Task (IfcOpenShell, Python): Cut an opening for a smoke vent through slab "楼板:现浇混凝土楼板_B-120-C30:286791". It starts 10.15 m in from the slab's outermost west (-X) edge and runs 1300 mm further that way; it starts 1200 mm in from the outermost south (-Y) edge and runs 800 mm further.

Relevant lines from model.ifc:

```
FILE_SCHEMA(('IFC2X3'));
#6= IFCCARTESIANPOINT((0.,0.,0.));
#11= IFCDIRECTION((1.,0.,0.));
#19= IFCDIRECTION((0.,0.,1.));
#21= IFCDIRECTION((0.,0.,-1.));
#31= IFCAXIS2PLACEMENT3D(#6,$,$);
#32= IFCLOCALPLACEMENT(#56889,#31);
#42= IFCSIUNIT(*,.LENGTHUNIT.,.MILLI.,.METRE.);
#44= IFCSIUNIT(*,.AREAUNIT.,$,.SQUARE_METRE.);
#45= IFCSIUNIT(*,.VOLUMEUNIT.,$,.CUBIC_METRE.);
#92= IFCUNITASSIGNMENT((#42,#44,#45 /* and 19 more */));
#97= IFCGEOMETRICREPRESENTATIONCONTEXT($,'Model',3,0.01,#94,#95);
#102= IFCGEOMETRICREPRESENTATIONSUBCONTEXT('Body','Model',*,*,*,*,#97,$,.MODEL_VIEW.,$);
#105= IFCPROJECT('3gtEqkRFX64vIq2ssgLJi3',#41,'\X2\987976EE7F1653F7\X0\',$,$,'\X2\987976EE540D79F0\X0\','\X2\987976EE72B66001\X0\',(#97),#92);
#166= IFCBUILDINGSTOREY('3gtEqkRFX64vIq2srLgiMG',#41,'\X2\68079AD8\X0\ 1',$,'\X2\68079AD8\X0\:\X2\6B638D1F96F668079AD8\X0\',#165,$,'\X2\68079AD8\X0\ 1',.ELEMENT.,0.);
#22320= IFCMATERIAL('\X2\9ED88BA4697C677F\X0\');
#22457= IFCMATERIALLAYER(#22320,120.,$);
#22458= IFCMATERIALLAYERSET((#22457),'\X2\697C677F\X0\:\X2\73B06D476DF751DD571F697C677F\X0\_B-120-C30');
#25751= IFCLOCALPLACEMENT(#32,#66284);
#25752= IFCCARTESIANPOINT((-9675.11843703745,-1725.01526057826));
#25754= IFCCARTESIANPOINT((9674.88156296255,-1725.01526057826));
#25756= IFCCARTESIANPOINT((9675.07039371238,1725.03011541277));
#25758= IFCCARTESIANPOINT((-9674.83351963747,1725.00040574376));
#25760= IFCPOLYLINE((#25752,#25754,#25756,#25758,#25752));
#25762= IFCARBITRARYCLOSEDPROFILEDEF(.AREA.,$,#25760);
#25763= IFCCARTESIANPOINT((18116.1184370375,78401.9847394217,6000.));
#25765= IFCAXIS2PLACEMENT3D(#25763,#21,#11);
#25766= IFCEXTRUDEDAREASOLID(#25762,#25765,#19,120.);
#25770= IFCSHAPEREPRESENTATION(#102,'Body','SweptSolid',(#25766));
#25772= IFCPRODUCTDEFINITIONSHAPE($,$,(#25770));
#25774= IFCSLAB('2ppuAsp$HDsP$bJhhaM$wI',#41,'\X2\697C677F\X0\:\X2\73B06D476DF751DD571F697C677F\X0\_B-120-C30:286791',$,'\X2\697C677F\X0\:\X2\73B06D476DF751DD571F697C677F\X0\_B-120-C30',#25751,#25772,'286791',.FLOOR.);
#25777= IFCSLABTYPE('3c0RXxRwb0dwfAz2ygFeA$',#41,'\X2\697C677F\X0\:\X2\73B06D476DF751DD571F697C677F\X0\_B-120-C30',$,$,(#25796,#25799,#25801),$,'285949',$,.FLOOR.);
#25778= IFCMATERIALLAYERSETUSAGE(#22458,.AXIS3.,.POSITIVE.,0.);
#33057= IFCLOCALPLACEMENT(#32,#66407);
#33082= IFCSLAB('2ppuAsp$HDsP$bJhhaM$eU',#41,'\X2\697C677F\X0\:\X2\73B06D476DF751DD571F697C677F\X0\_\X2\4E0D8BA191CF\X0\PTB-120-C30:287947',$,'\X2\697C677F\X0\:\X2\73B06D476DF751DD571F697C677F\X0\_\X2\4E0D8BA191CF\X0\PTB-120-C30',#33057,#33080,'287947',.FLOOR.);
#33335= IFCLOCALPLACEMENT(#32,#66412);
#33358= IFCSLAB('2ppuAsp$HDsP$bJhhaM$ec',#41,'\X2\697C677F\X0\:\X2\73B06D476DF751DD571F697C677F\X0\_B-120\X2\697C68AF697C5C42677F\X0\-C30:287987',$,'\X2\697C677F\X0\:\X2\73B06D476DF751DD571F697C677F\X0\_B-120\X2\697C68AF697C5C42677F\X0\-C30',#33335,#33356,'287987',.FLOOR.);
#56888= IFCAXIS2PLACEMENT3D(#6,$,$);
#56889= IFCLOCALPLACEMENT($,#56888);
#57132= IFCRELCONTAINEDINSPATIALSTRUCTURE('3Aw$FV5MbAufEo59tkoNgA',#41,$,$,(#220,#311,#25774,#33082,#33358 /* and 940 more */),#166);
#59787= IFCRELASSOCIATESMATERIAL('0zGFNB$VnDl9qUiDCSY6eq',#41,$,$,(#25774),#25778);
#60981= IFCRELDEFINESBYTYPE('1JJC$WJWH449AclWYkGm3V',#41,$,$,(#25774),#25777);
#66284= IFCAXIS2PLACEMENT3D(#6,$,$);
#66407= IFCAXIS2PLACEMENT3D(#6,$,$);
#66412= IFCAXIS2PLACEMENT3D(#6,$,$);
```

```python
import numpy as np
import ifcopenshell
import ifcopenshell.api.feature
import ifcopenshell.api.geometry
import ifcopenshell.api.root
import ifcopenshell.geom
import ifcopenshell.util.placement
import ifcopenshell.util.representation
import ifcopenshell.util.shape
import ifcopenshell.util.unit

model = ifcopenshell.open("model.ifc")
unit_scale = ifcopenshell.util.unit.calculate_unit_scale(model)
settings = ifcopenshell.geom.settings()


def volume(element):
    """Net volume in cubic metres, openings subtracted."""
    shape = ifcopenshell.geom.create_shape(settings, element)
    return ifcopenshell.util.shape.get_volume(shape.geometry)


slab = model.by_guid("2ppuAsp$HDsP$bJhhaM$wI")
before = volume(slab)

# Extent in the slab's own axes, in metres. The edges named are its -X and -Y sides.
slab_shape = ifcopenshell.geom.create_shape(settings, slab)
vertices = ifcopenshell.util.shape.get_vertices(slab_shape.geometry)
x_min, y_min, bottom = vertices.min(axis=0)
top = vertices[:, 2].max()

opening = ifcopenshell.api.root.create_entity(model, ifc_class="IfcOpeningElement", name="Smoke vent opening")
context = ifcopenshell.util.representation.get_context(model, "Model", "Body", "MODEL_VIEW")
width, depth = 1.3, 0.8
outline = [(0.0, 0.0), (width, 0.0), (width, depth), (0.0, depth), (0.0, 0.0)]
# Overshoot both faces by 50 mm so the cut is clean.
shape = ifcopenshell.api.geometry.add_slab_representation(
    model, context=context, depth=top - bottom + 0.1, polyline=outline
)
ifcopenshell.api.geometry.assign_representation(model, product=opening, representation=shape)

matrix = ifcopenshell.util.placement.get_local_placement(slab.ObjectPlacement)
matrix[:, 3] = matrix @ np.append(np.array([x_min + 10.15, y_min + 1.2, bottom - 0.05]) / unit_scale, 1.0)
ifcopenshell.api.geometry.edit_object_placement(model, product=opening, matrix=matrix, is_si=False)
ifcopenshell.api.feature.add_feature(model, feature=opening, element=slab)

after = volume(slab)

print(f"slab volume {before:.3f} -> {after:.3f} m3")

model.write("model_rev.ifc")
```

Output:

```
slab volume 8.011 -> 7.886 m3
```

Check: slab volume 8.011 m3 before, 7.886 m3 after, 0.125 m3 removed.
